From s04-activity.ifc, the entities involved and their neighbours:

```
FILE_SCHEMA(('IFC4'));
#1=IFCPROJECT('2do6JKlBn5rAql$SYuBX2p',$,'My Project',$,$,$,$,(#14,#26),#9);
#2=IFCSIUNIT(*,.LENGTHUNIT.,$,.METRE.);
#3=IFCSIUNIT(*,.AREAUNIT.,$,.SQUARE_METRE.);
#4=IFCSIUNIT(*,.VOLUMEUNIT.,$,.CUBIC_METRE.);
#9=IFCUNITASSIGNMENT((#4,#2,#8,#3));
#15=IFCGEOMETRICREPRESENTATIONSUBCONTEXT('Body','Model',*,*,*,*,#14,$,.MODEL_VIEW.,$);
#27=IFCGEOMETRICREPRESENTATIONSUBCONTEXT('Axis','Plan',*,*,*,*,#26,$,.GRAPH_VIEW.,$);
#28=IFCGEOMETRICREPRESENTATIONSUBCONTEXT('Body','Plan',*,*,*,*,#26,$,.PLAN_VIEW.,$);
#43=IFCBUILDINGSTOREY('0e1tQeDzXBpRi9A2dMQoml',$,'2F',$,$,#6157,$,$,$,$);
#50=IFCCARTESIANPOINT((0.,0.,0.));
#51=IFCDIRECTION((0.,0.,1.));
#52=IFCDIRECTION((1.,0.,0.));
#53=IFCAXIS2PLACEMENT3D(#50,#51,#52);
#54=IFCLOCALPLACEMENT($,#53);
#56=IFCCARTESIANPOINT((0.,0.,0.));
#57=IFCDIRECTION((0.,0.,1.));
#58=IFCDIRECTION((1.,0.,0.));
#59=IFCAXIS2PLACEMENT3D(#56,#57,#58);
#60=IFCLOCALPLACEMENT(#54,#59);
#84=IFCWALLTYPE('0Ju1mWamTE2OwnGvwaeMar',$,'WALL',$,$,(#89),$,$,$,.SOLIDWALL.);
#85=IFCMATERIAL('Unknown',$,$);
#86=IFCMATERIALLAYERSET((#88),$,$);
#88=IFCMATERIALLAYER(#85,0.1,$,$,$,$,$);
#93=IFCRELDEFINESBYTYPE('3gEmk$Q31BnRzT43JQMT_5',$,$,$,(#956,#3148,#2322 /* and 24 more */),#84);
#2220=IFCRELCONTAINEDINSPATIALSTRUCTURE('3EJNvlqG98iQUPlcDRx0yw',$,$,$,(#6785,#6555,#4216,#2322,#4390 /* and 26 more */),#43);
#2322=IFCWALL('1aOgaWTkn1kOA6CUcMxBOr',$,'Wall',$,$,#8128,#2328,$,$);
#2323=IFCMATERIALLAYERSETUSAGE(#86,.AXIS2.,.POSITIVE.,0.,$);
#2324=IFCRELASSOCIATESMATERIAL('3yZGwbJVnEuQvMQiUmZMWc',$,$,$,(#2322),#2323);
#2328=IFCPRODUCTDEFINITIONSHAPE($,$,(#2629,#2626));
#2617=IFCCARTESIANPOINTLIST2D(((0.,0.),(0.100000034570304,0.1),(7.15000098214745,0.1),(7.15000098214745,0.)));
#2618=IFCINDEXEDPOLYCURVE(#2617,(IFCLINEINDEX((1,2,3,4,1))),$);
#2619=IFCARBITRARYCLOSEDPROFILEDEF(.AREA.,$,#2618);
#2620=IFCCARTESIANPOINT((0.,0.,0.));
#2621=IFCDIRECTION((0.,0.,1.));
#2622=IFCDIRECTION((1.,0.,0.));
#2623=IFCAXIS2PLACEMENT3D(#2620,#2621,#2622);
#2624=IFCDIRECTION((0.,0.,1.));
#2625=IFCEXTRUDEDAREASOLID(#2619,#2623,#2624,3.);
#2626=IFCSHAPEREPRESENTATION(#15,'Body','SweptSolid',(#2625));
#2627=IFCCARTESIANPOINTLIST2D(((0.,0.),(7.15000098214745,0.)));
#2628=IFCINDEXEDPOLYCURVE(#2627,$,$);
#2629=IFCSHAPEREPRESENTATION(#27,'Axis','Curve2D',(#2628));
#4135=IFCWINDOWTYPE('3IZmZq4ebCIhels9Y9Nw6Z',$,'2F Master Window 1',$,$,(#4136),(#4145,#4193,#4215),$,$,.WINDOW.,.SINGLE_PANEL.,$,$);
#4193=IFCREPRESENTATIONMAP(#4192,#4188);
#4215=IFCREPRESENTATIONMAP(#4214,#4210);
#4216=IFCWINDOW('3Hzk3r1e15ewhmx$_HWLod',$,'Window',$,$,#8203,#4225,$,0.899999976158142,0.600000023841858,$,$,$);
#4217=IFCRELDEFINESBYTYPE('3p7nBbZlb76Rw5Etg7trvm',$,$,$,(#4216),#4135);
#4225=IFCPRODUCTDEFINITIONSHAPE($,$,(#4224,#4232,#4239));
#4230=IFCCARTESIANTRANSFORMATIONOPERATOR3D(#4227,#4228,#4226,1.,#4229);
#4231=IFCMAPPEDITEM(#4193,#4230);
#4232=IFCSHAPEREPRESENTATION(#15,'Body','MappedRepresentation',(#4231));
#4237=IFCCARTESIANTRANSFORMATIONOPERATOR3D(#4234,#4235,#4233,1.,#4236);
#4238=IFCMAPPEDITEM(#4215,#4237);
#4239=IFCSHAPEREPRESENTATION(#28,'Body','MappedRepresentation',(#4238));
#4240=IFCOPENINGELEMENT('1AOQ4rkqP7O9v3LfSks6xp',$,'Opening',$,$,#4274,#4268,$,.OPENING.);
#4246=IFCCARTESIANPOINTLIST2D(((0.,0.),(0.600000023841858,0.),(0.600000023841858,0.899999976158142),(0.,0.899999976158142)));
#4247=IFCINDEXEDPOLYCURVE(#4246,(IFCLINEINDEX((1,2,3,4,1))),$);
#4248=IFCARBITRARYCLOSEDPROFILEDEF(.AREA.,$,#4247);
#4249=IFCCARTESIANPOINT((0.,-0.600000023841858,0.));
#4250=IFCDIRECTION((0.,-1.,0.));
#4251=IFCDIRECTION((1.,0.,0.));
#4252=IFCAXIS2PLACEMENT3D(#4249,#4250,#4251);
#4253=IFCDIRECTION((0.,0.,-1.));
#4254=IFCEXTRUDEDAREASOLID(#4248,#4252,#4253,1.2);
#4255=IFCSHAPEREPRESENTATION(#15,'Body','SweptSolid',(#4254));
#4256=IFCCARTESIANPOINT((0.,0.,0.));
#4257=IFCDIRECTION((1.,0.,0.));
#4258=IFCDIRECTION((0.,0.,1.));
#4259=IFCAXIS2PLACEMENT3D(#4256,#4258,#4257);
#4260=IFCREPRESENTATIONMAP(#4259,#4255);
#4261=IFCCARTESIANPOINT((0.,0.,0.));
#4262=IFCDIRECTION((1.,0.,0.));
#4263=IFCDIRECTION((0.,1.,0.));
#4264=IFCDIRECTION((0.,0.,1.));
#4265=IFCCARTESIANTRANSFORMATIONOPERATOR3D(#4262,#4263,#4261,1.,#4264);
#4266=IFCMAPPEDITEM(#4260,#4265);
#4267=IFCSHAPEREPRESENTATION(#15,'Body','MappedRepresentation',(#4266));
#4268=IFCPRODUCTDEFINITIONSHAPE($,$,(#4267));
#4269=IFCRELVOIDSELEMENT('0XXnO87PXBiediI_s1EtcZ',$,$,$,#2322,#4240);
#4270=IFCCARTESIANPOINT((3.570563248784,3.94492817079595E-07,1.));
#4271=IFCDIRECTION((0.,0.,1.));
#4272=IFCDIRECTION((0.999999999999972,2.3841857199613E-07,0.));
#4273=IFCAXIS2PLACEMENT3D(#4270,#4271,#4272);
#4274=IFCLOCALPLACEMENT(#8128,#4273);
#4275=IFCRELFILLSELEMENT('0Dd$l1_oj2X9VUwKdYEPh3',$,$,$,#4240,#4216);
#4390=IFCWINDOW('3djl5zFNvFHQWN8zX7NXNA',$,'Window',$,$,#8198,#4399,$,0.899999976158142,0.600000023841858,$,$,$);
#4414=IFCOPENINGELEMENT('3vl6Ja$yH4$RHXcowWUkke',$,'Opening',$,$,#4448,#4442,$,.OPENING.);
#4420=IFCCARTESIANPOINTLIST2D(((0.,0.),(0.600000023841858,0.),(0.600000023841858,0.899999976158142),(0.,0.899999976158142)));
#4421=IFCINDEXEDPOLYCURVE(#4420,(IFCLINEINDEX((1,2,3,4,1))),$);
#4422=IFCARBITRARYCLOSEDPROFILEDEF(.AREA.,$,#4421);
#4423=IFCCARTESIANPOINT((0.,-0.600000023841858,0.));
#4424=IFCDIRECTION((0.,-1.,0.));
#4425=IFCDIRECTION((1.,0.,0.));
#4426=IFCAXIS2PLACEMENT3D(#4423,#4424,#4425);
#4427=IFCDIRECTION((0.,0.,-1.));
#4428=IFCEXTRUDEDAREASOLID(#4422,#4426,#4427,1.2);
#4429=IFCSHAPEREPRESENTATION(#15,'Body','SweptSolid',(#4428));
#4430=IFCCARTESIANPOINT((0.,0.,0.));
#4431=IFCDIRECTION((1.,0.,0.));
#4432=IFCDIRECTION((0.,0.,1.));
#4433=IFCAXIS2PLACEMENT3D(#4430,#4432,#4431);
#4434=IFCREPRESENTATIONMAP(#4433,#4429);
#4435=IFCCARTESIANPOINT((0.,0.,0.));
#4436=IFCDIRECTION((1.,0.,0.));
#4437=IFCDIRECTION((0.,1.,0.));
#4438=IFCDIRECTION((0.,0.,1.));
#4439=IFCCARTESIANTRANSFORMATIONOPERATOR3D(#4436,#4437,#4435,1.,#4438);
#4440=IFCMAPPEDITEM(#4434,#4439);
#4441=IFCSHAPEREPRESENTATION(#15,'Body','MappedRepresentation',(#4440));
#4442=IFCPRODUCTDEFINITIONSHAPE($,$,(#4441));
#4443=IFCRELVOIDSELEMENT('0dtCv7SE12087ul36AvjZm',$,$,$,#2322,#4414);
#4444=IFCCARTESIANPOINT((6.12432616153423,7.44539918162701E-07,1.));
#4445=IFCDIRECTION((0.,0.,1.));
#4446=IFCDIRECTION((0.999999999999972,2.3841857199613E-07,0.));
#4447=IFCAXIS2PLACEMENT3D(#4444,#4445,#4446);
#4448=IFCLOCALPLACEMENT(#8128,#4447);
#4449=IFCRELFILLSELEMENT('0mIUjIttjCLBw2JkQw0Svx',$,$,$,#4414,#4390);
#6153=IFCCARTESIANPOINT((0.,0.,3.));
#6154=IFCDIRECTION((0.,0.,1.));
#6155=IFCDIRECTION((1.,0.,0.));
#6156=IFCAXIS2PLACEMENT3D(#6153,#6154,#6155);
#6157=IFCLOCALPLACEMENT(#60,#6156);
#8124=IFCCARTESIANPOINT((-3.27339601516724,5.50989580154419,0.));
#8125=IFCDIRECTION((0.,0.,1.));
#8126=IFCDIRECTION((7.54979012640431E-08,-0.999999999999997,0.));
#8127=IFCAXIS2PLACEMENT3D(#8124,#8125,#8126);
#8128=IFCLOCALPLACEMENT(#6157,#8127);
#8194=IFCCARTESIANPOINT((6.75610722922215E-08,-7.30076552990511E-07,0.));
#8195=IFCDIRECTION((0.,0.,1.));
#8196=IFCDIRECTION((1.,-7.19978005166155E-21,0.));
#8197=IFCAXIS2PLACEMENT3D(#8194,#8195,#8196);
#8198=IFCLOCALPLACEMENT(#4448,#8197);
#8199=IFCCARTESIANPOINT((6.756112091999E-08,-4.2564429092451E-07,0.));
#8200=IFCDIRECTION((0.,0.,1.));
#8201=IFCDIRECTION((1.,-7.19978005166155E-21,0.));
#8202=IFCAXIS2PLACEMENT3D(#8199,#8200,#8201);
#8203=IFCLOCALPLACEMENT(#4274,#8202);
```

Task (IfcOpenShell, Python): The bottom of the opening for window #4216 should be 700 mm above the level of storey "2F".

```python
import numpy as np
import ifcopenshell
import ifcopenshell.api.geometry
import ifcopenshell.geom
import ifcopenshell.util.element
import ifcopenshell.util.placement
import ifcopenshell.util.shape
import ifcopenshell.util.unit

model = ifcopenshell.open("s04-activity.ifc")
unit_scale = ifcopenshell.util.unit.calculate_unit_scale(model)

window = model.by_id(4216)
opening = window.FillsVoids[0].RelatingOpeningElement
storey = ifcopenshell.util.element.get_container(window, ifc_class="IfcBuildingStorey")
level = ifcopenshell.util.placement.get_local_placement(storey.ObjectPlacement)[2, 3]

# The opening's origin need not be at the sill, so measure its lowest point.
shape = ifcopenshell.geom.create_shape(ifcopenshell.geom.settings(), opening)
bottom = ifcopenshell.util.shape.get_shape_bottom_elevation(shape, shape.geometry) / unit_scale
dz = level + 0.7 - bottom

shift = np.array([0.0, 0.0, dz])
# The window is placed relative to its opening, so it follows when the opening moves.
matrix = ifcopenshell.util.placement.get_local_placement(opening.ObjectPlacement)
matrix[:3, 3] += shift
ifcopenshell.api.geometry.edit_object_placement(
    model, product=opening, matrix=matrix, is_si=False, should_transform_children=True
)

print(f"moved by {dz * unit_scale:+.3f} m")

model.write("s04-activity-out.ifc")
```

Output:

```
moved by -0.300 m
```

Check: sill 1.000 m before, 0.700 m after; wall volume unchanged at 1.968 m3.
